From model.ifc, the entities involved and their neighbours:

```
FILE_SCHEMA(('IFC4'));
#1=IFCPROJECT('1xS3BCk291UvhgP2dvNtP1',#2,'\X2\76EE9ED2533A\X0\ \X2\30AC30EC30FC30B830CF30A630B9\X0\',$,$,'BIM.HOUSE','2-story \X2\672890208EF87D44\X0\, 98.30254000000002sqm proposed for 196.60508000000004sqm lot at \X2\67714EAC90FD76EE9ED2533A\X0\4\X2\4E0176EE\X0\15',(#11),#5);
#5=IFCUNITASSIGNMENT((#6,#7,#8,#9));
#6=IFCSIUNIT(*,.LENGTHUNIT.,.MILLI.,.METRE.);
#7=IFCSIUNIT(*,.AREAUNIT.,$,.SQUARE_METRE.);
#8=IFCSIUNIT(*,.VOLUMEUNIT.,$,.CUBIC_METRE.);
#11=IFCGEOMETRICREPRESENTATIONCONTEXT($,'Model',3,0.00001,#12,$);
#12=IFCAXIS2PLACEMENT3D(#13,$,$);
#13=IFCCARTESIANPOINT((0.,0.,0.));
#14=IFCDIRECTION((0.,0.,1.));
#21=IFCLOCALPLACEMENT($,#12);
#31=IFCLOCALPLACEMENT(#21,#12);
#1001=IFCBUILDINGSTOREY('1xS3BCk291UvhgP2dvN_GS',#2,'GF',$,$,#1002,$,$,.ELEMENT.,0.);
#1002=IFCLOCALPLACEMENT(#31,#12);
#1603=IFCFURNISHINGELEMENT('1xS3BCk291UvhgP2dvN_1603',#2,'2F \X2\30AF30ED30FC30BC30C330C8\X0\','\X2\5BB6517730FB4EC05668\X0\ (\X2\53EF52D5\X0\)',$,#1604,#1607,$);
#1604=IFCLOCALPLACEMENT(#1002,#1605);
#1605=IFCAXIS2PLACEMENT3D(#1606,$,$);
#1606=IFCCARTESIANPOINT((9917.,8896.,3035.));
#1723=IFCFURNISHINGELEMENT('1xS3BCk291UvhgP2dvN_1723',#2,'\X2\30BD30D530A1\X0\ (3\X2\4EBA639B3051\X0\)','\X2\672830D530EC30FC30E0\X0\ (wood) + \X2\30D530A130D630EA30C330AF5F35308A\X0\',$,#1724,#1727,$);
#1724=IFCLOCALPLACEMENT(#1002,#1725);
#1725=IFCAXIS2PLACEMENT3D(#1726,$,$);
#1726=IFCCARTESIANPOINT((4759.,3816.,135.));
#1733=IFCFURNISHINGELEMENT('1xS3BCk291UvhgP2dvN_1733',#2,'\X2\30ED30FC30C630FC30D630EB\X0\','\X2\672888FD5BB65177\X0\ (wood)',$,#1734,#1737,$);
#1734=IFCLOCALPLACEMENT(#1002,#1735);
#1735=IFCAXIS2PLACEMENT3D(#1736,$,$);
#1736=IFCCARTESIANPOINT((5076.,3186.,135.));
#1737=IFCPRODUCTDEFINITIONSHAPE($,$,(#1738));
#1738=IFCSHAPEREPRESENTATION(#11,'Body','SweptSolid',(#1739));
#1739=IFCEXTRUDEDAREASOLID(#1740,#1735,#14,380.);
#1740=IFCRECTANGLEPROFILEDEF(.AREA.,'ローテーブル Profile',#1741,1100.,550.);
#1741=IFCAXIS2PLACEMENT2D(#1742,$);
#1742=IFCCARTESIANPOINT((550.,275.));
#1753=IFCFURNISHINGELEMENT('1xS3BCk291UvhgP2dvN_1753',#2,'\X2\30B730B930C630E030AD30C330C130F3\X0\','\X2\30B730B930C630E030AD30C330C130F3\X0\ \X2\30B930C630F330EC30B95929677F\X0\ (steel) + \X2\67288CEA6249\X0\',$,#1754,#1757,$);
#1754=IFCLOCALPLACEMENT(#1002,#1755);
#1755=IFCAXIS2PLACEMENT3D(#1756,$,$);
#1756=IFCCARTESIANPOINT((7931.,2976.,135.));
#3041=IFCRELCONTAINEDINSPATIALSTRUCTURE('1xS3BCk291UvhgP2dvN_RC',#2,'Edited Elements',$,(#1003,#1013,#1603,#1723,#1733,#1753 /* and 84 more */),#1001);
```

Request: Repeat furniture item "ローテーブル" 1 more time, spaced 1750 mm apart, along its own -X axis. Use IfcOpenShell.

```python
import ifcopenshell
import ifcopenshell.api.geometry
import ifcopenshell.api.root
import ifcopenshell.util.element
import ifcopenshell.util.placement
import ifcopenshell.util.unit

model = ifcopenshell.open("model.ifc")
unit_scale = ifcopenshell.util.unit.calculate_unit_scale(model)


def reuse_history(source, copy):
    """copy_class also copies each property set's owner history, people and application; keep the originals."""
    for rel in copy.IsDefinedBy:
        if rel.is_a("IfcRelDefinesByProperties") and (history := rel.RelatingPropertyDefinition.OwnerHistory):
            rel.RelatingPropertyDefinition.OwnerHistory = source.OwnerHistory
            ifcopenshell.util.element.remove_deep2(model, history)


source = model.by_guid("1xS3BCk291UvhgP2dvN_1733")
base = ifcopenshell.util.placement.get_local_placement(source.ObjectPlacement)
step = -base[:3, 0] * 1.75 / unit_scale

for i in range(1, 2):
    copy = ifcopenshell.api.root.copy_class(model, product=source)
    copy.Representation = ifcopenshell.util.element.copy_deep(
        model, source.Representation, exclude=["IfcGeometricRepresentationContext", "IfcRepresentationMap"]
    )
    reuse_history(source, copy)
    matrix = base.copy()
    matrix[:3, 3] += i * step
    print("added at", matrix[:3, 3].round(3) + 0.0)
    ifcopenshell.api.geometry.edit_object_placement(model, product=copy, matrix=matrix, is_si=False)

model.write("model-out.ifc")
```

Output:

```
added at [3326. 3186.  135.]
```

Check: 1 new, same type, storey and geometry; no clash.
